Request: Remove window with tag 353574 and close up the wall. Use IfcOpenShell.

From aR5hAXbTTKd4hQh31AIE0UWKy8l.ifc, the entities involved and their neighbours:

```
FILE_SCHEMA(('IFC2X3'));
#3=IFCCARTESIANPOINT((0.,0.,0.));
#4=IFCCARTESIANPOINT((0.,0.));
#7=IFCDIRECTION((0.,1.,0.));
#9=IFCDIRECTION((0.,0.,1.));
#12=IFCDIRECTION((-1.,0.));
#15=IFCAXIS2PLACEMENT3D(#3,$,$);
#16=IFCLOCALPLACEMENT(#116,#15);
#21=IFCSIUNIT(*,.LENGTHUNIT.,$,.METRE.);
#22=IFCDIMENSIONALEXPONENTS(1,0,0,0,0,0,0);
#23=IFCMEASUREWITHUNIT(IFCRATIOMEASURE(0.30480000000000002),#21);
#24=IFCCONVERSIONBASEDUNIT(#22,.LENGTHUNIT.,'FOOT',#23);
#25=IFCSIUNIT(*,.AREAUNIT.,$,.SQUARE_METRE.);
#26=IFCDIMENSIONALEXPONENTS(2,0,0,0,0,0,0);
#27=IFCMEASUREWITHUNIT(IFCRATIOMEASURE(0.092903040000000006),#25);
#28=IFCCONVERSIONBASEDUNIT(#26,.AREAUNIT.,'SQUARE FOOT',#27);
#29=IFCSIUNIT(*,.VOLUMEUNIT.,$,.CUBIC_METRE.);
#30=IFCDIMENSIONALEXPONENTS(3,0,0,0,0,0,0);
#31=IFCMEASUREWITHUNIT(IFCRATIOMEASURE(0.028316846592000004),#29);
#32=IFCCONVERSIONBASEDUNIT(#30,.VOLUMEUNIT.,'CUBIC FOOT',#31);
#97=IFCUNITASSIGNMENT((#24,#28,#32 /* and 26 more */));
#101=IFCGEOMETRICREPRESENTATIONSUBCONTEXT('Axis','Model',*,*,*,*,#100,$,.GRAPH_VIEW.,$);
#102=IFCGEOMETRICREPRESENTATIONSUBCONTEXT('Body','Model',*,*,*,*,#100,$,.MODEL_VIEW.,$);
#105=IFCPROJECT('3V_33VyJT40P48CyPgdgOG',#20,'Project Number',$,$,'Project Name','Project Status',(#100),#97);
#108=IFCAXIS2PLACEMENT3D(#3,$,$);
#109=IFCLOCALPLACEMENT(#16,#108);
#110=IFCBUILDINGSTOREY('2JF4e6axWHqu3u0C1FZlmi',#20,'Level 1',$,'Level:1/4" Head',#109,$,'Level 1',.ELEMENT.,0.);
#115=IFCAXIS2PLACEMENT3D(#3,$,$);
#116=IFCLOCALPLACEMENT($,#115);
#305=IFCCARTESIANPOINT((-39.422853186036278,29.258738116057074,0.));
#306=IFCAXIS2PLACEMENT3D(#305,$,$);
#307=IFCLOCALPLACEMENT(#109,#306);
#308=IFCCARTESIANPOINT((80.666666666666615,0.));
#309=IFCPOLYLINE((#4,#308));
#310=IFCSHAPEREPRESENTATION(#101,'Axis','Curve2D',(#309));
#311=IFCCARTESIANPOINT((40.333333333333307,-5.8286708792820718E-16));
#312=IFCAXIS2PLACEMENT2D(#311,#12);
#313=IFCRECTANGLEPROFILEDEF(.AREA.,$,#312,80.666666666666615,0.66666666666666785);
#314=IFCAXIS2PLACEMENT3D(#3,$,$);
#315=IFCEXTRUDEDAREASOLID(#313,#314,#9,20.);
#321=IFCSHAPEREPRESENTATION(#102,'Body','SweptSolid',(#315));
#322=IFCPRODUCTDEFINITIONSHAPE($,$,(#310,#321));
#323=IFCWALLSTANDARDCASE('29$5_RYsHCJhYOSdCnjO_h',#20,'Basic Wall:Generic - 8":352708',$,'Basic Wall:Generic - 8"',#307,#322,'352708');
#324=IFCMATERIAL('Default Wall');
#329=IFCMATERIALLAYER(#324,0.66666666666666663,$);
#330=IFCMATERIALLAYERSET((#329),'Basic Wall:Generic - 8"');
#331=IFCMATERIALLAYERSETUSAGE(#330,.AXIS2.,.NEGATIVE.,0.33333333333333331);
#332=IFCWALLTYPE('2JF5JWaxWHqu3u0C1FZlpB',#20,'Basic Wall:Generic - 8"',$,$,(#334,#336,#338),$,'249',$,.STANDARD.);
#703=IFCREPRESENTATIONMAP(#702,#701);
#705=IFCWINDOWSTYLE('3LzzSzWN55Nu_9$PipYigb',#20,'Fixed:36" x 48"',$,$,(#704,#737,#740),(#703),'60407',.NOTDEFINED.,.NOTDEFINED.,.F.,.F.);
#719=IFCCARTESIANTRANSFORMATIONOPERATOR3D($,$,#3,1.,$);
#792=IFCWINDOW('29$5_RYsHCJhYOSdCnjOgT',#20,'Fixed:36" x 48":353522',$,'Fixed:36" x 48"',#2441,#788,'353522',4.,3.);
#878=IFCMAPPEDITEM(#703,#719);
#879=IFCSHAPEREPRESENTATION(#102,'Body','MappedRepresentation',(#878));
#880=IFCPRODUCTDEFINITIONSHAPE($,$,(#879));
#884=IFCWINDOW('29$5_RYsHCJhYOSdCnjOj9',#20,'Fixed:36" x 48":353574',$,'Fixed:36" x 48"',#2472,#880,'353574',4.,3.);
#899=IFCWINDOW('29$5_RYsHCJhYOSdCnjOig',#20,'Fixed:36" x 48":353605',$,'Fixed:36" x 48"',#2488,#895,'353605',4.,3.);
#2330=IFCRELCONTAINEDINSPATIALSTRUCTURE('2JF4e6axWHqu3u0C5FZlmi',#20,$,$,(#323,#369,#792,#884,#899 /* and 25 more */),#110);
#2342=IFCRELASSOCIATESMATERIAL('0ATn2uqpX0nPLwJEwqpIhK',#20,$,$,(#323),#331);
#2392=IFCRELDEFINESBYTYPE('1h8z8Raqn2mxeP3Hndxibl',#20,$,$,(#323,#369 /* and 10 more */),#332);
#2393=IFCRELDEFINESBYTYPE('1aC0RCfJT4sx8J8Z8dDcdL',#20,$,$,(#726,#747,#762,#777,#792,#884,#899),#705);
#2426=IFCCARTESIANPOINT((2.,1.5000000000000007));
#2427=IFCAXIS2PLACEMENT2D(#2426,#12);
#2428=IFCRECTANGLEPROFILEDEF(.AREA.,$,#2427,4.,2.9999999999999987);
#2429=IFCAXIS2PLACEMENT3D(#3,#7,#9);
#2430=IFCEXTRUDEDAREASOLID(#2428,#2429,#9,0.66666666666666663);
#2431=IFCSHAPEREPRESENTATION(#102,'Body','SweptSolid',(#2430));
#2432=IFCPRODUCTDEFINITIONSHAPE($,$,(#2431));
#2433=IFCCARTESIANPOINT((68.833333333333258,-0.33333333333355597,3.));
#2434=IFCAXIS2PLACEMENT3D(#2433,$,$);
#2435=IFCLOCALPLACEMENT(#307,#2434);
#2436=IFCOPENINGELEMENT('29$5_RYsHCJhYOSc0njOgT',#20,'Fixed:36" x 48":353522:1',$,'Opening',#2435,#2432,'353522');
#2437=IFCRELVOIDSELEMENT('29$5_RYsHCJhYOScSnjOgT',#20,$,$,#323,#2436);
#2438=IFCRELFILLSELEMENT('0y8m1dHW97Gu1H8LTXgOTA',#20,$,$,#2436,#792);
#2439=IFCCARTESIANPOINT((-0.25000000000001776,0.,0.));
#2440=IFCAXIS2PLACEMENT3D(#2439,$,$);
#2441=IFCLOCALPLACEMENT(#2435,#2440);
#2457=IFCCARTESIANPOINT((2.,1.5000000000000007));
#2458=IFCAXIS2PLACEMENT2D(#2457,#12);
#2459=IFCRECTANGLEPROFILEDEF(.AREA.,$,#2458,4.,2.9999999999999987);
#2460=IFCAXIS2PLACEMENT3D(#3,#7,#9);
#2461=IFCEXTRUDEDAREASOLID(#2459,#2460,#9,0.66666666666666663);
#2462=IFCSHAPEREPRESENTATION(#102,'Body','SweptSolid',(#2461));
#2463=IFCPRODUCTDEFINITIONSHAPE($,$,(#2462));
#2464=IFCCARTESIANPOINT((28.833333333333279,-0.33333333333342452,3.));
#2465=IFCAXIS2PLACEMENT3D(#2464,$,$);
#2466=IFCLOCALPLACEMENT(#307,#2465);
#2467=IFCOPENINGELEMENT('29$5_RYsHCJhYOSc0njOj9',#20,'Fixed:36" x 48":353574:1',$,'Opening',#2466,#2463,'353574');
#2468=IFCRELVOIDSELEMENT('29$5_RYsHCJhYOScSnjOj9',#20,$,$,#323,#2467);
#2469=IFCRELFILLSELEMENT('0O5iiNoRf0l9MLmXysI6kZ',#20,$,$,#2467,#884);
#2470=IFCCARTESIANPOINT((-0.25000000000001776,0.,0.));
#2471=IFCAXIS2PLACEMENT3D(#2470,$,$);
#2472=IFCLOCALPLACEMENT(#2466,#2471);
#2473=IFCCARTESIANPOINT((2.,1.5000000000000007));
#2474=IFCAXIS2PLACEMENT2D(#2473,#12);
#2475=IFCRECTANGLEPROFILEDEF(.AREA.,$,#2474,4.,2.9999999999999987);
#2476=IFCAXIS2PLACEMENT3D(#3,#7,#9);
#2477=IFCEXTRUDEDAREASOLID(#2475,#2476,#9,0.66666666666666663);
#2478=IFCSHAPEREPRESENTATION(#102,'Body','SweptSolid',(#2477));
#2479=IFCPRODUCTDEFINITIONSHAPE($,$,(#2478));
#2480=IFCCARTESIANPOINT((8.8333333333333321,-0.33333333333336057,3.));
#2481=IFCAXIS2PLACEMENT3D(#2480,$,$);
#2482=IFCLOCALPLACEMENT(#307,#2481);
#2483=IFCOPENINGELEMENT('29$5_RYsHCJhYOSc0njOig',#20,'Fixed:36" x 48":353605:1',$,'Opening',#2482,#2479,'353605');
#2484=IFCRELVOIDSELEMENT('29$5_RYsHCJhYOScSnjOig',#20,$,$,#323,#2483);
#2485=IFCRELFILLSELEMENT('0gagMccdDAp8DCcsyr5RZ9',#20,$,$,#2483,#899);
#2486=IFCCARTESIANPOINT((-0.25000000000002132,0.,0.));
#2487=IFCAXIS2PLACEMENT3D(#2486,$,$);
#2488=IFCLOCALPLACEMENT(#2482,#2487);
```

```python
import ifcopenshell
import ifcopenshell.api.feature
import ifcopenshell.api.root
import ifcopenshell.geom
import ifcopenshell.util.shape

model = ifcopenshell.open("aR5hAXbTTKd4hQh31AIE0UWKy8l.ifc")
settings = ifcopenshell.geom.settings()


def volume(element):
    """Net volume in cubic metres, openings subtracted."""
    shape = ifcopenshell.geom.create_shape(settings, element)
    return ifcopenshell.util.shape.get_volume(shape.geometry)


window = model.by_guid("29$5_RYsHCJhYOSdCnjOj9")
opening = window.FillsVoids[0].RelatingOpeningElement
wall = opening.VoidsElements[0].RelatingBuildingElement
before = volume(wall)

ifcopenshell.api.root.remove_product(model, product=window)
ifcopenshell.api.feature.remove_feature(model, feature=opening)

after = volume(wall)

print(f"wall volume {before:.3f} -> {after:.3f} m3")

model.write("aR5hAXbTTKd4hQh31AIE0UWKy8l-out.ifc")
```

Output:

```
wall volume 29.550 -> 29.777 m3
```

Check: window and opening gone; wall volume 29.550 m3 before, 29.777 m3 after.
